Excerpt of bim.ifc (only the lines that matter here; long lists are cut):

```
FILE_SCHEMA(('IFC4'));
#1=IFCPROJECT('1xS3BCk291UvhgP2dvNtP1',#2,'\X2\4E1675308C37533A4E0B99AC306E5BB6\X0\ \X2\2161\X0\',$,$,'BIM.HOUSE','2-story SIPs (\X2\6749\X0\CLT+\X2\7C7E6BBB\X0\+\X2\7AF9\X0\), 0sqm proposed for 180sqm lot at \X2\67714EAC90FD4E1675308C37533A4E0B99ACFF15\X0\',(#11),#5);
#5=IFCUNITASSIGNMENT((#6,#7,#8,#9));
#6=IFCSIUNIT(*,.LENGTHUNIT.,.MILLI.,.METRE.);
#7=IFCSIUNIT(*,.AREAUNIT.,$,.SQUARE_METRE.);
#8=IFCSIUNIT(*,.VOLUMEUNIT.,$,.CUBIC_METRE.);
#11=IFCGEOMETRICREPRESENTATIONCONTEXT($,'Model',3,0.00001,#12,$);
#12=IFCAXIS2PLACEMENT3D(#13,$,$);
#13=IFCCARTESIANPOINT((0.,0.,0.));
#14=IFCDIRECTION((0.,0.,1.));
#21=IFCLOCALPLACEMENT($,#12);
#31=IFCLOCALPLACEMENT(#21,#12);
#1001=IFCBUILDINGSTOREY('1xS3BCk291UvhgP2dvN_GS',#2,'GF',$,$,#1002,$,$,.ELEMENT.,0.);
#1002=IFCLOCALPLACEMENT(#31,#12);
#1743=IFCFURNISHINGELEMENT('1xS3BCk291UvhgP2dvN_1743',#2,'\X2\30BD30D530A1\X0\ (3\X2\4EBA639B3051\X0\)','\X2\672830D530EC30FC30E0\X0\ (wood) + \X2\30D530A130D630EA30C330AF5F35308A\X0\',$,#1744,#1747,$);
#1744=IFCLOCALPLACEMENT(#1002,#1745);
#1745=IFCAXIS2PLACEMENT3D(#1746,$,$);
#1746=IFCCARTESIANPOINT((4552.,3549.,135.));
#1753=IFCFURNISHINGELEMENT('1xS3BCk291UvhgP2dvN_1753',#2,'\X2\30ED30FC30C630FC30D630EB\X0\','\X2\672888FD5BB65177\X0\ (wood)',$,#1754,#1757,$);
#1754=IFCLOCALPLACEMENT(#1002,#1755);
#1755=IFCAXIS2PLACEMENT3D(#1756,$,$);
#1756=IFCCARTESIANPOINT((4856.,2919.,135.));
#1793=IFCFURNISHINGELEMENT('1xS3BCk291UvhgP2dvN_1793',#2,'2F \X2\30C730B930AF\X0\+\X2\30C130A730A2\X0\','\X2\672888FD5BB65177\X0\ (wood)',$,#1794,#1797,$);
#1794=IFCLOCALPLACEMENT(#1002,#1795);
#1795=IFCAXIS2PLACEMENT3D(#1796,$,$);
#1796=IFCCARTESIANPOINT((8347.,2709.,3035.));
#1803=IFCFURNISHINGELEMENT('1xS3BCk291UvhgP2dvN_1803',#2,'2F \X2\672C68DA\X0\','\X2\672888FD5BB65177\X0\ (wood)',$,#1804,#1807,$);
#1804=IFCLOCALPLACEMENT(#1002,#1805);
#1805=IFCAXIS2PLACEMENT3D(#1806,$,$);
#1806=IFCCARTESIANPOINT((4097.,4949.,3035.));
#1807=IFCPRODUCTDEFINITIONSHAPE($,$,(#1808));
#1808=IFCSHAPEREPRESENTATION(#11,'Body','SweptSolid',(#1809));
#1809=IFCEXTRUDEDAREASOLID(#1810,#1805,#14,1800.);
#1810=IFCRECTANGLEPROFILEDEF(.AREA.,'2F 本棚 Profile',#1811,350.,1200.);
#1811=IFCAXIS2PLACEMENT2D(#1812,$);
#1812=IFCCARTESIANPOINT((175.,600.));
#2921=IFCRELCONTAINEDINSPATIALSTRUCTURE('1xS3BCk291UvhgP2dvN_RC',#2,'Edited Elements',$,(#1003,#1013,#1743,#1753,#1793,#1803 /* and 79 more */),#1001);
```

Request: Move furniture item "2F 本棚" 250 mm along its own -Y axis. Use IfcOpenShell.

```python
import ifcopenshell
import ifcopenshell.api.geometry
import ifcopenshell.util.placement
import ifcopenshell.util.unit

model = ifcopenshell.open("bim.ifc")
unit_scale = ifcopenshell.util.unit.calculate_unit_scale(model)

item = model.by_id(1803)
matrix = ifcopenshell.util.placement.get_local_placement(item.ObjectPlacement)
matrix[:3, 3] -= matrix[:3, 1] * 0.25 / unit_scale
ifcopenshell.api.geometry.edit_object_placement(model, product=item, matrix=matrix, is_si=False)

print(ifcopenshell.util.placement.get_local_placement(item.ObjectPlacement).round(3) + 0.0)

model.write("bim_v2.ifc")
```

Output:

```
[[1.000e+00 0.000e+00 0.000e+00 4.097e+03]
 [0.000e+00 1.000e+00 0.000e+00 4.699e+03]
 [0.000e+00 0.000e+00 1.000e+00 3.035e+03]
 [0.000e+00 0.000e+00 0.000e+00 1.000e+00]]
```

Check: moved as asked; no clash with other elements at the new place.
